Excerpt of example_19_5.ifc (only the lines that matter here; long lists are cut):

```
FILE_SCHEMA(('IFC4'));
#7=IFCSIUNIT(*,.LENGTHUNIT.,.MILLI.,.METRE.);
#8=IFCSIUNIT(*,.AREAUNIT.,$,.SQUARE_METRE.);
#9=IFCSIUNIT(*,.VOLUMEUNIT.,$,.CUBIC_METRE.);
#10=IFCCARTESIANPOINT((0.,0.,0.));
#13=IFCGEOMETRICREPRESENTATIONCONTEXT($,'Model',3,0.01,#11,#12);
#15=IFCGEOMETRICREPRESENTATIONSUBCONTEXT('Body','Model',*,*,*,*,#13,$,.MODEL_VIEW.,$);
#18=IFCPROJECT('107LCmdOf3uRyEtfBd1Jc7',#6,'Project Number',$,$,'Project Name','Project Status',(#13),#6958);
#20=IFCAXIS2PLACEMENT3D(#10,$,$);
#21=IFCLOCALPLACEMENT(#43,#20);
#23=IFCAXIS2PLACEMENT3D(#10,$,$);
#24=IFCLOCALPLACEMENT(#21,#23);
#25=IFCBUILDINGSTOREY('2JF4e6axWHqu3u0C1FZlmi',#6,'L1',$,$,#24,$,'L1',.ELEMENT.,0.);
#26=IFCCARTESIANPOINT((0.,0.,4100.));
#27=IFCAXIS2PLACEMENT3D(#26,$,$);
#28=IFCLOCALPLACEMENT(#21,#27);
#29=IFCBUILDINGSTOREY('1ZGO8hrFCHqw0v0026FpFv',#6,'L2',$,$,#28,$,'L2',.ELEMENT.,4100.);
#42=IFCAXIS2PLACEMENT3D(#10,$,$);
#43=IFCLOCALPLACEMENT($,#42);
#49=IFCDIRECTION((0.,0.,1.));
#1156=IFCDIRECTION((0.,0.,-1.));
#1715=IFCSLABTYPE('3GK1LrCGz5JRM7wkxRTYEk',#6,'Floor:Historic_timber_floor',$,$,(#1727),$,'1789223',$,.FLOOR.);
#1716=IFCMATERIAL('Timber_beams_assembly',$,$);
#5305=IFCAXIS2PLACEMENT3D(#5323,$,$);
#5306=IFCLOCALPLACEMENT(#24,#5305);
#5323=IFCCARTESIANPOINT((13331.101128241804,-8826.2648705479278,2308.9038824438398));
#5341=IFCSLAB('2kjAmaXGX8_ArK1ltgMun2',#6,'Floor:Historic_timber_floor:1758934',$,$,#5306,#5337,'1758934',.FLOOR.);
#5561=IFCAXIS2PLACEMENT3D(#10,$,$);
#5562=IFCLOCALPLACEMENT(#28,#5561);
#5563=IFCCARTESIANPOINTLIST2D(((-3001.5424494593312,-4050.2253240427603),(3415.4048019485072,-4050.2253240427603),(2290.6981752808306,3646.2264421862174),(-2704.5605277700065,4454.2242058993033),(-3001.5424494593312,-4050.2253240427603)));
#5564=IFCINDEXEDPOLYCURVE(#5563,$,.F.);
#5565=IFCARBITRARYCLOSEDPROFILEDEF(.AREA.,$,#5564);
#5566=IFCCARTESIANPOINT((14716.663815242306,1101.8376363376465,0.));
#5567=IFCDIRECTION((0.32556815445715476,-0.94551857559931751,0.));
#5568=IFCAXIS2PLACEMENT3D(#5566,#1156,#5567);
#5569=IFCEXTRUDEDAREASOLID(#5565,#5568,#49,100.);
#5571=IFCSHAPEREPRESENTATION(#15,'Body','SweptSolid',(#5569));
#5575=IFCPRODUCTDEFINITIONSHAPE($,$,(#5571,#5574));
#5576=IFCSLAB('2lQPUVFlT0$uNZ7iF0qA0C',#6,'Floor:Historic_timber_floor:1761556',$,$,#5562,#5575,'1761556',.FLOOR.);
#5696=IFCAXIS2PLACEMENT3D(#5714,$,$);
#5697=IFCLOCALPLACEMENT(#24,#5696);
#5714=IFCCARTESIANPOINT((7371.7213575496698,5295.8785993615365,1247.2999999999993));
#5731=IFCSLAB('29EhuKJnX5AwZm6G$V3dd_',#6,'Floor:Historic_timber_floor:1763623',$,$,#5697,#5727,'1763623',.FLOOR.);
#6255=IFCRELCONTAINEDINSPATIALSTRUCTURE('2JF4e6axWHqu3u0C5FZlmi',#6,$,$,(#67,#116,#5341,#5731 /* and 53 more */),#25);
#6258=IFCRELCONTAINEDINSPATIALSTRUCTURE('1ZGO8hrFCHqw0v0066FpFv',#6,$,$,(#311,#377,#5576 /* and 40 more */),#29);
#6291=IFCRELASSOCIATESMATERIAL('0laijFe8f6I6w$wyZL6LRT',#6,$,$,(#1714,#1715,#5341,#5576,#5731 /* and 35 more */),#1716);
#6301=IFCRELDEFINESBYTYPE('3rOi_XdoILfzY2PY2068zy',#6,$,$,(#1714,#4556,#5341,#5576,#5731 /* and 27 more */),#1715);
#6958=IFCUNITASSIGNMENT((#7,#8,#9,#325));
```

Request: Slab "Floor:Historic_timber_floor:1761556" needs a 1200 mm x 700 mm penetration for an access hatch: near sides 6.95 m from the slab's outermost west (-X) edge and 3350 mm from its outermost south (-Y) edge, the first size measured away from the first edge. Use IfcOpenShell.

```python
import numpy as np
import ifcopenshell
import ifcopenshell.api.feature
import ifcopenshell.api.geometry
import ifcopenshell.api.root
import ifcopenshell.geom
import ifcopenshell.util.placement
import ifcopenshell.util.representation
import ifcopenshell.util.shape
import ifcopenshell.util.unit

model = ifcopenshell.open("example_19_5.ifc")
unit_scale = ifcopenshell.util.unit.calculate_unit_scale(model)
settings = ifcopenshell.geom.settings()


def volume(element):
    """Net volume in cubic metres, openings subtracted."""
    shape = ifcopenshell.geom.create_shape(settings, element)
    return ifcopenshell.util.shape.get_volume(shape.geometry)


slab = model.by_guid("2lQPUVFlT0$uNZ7iF0qA0C")
before = volume(slab)

# Extent in the slab's own axes, in metres. The edges named are its -X and -Y sides.
slab_shape = ifcopenshell.geom.create_shape(settings, slab)
vertices = ifcopenshell.util.shape.get_vertices(slab_shape.geometry)
x_min, y_min, bottom = vertices.min(axis=0)
top = vertices[:, 2].max()

opening = ifcopenshell.api.root.create_entity(model, ifc_class="IfcOpeningElement", name="Access hatch opening", predefined_type="OPENING")
context = ifcopenshell.util.representation.get_context(model, "Model", "Body", "MODEL_VIEW")
width, depth = 1.2, 0.7
outline = [(0.0, 0.0), (width, 0.0), (width, depth), (0.0, depth), (0.0, 0.0)]
# Overshoot both faces by 50 mm so the cut is clean.
shape = ifcopenshell.api.geometry.add_slab_representation(
    model, context=context, depth=top - bottom + 0.1, polyline=outline
)
ifcopenshell.api.geometry.assign_representation(model, product=opening, representation=shape)

matrix = ifcopenshell.util.placement.get_local_placement(slab.ObjectPlacement)
matrix[:, 3] = matrix @ np.append(np.array([x_min + 6.95, y_min + 3.35, bottom - 0.05]) / unit_scale, 1.0)
ifcopenshell.api.geometry.edit_object_placement(model, product=opening, matrix=matrix, is_si=False)
ifcopenshell.api.feature.add_feature(model, feature=opening, element=slab)

after = volume(slab)

print(f"slab volume {before:.3f} -> {after:.3f} m3")

model.write("example_19_5-out.ifc")
```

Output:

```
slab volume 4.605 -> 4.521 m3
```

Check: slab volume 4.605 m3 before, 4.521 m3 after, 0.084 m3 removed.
